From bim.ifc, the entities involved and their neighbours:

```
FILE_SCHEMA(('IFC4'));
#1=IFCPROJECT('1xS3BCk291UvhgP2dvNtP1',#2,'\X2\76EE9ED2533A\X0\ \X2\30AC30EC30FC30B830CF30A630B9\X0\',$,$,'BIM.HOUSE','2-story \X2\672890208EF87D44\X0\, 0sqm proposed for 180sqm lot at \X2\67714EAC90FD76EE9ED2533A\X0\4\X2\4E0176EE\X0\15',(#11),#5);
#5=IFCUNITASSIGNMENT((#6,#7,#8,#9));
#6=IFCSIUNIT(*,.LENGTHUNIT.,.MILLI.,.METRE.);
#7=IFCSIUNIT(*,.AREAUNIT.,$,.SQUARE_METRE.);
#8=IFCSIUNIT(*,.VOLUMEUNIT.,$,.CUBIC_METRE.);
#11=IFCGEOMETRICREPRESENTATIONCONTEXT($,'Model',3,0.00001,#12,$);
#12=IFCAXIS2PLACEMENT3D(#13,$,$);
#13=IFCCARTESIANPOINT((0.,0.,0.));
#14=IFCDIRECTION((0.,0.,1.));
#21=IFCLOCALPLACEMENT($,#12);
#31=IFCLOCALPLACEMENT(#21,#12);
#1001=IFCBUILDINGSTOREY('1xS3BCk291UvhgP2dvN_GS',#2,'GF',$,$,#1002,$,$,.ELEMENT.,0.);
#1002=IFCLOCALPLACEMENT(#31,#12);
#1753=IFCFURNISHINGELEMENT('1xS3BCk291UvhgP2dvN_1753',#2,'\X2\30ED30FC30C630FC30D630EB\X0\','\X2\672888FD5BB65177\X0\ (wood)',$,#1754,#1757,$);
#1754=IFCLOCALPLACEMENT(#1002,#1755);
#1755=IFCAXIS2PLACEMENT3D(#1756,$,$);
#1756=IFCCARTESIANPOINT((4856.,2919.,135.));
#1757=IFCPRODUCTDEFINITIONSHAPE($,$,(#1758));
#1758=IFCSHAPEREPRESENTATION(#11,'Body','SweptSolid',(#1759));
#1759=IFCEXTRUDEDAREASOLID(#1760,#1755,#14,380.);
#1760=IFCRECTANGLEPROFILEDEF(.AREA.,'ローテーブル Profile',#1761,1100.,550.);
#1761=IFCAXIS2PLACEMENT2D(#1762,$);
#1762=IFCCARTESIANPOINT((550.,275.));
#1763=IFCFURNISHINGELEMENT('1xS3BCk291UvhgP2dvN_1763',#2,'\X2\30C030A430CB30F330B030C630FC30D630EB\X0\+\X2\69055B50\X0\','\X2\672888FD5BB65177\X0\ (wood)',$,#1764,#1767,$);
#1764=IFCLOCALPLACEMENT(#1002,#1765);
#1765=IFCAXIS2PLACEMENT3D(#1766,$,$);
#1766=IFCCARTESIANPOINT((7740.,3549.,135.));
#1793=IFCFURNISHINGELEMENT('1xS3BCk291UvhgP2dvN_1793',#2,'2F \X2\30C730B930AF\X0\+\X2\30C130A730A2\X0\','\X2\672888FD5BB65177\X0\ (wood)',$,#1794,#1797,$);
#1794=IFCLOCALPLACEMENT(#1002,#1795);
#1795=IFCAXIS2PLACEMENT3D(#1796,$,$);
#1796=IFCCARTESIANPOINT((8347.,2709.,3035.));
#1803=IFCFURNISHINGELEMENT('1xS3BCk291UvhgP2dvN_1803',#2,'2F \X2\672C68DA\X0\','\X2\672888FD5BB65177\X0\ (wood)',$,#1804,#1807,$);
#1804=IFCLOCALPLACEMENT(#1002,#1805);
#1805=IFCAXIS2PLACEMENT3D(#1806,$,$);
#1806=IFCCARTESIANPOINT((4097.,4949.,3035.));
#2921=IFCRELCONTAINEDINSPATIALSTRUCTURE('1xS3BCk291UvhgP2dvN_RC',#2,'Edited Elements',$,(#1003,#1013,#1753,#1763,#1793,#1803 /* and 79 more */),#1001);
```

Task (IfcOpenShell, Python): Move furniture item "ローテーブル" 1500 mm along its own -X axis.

```python
import ifcopenshell
import ifcopenshell.api.geometry
import ifcopenshell.util.placement
import ifcopenshell.util.unit

model = ifcopenshell.open("bim.ifc")
unit_scale = ifcopenshell.util.unit.calculate_unit_scale(model)

item = model.by_guid("1xS3BCk291UvhgP2dvN_1753")
matrix = ifcopenshell.util.placement.get_local_placement(item.ObjectPlacement)
matrix[:3, 3] -= matrix[:3, 0] * 1.5 / unit_scale
ifcopenshell.api.geometry.edit_object_placement(model, product=item, matrix=matrix, is_si=False)

print(ifcopenshell.util.placement.get_local_placement(item.ObjectPlacement).round(3) + 0.0)

model.write("bim-out.ifc")
```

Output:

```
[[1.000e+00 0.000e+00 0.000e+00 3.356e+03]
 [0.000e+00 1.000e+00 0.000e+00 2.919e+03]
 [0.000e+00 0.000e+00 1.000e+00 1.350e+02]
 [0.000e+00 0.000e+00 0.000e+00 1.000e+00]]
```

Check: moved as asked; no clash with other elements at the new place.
